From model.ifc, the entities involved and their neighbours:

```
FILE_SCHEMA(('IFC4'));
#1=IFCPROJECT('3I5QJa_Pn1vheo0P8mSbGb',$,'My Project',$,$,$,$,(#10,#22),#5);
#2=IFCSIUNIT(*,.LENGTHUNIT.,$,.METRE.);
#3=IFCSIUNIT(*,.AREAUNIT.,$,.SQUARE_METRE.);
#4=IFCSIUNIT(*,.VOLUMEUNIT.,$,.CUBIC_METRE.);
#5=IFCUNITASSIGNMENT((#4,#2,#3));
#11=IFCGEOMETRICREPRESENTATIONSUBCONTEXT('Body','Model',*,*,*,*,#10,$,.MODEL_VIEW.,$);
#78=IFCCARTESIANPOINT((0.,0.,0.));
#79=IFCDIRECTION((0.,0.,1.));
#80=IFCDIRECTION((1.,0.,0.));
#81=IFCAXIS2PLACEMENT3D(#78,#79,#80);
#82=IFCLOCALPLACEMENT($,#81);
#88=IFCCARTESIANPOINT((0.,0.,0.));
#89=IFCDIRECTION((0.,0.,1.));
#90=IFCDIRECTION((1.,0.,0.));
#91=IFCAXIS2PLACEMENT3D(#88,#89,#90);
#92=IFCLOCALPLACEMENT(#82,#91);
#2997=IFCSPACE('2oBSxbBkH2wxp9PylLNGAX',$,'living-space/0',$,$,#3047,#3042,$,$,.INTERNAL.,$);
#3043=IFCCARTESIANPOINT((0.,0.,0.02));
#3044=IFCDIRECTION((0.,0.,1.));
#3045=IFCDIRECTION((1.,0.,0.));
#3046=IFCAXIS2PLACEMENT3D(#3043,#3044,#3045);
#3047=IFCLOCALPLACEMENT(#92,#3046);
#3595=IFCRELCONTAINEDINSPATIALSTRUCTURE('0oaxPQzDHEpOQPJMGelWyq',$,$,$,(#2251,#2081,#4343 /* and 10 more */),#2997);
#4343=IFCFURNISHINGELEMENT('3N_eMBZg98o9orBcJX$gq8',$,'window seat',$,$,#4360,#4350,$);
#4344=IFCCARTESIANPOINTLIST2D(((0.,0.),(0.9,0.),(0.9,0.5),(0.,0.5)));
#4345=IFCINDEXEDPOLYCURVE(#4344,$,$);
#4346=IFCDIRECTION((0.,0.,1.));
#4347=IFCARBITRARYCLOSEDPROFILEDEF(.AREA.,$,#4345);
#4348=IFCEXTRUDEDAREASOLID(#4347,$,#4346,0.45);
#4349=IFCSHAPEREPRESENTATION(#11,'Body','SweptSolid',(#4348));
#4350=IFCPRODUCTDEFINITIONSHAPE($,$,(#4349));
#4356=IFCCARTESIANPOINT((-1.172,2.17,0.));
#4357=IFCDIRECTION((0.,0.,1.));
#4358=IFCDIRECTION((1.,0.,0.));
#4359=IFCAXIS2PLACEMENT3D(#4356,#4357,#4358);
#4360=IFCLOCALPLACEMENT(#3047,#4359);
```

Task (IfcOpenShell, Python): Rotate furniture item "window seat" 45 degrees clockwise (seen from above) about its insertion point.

```python
import ifcopenshell
import ifcopenshell.api.geometry
import ifcopenshell.util.placement

model = ifcopenshell.open("model.ifc")

item = model.by_guid("3N_eMBZg98o9orBcJX$gq8")
matrix = ifcopenshell.util.placement.get_local_placement(item.ObjectPlacement)
matrix = matrix @ ifcopenshell.util.placement.rotation(-45, "Z")
ifcopenshell.api.geometry.edit_object_placement(model, product=item, matrix=matrix, is_si=False)

print(ifcopenshell.util.placement.get_local_placement(item.ObjectPlacement).round(3) + 0.0)

model.write("model-out.ifc")
```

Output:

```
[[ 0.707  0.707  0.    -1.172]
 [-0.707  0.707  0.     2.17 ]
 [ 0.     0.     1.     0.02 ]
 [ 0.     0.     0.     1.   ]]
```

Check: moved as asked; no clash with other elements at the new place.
